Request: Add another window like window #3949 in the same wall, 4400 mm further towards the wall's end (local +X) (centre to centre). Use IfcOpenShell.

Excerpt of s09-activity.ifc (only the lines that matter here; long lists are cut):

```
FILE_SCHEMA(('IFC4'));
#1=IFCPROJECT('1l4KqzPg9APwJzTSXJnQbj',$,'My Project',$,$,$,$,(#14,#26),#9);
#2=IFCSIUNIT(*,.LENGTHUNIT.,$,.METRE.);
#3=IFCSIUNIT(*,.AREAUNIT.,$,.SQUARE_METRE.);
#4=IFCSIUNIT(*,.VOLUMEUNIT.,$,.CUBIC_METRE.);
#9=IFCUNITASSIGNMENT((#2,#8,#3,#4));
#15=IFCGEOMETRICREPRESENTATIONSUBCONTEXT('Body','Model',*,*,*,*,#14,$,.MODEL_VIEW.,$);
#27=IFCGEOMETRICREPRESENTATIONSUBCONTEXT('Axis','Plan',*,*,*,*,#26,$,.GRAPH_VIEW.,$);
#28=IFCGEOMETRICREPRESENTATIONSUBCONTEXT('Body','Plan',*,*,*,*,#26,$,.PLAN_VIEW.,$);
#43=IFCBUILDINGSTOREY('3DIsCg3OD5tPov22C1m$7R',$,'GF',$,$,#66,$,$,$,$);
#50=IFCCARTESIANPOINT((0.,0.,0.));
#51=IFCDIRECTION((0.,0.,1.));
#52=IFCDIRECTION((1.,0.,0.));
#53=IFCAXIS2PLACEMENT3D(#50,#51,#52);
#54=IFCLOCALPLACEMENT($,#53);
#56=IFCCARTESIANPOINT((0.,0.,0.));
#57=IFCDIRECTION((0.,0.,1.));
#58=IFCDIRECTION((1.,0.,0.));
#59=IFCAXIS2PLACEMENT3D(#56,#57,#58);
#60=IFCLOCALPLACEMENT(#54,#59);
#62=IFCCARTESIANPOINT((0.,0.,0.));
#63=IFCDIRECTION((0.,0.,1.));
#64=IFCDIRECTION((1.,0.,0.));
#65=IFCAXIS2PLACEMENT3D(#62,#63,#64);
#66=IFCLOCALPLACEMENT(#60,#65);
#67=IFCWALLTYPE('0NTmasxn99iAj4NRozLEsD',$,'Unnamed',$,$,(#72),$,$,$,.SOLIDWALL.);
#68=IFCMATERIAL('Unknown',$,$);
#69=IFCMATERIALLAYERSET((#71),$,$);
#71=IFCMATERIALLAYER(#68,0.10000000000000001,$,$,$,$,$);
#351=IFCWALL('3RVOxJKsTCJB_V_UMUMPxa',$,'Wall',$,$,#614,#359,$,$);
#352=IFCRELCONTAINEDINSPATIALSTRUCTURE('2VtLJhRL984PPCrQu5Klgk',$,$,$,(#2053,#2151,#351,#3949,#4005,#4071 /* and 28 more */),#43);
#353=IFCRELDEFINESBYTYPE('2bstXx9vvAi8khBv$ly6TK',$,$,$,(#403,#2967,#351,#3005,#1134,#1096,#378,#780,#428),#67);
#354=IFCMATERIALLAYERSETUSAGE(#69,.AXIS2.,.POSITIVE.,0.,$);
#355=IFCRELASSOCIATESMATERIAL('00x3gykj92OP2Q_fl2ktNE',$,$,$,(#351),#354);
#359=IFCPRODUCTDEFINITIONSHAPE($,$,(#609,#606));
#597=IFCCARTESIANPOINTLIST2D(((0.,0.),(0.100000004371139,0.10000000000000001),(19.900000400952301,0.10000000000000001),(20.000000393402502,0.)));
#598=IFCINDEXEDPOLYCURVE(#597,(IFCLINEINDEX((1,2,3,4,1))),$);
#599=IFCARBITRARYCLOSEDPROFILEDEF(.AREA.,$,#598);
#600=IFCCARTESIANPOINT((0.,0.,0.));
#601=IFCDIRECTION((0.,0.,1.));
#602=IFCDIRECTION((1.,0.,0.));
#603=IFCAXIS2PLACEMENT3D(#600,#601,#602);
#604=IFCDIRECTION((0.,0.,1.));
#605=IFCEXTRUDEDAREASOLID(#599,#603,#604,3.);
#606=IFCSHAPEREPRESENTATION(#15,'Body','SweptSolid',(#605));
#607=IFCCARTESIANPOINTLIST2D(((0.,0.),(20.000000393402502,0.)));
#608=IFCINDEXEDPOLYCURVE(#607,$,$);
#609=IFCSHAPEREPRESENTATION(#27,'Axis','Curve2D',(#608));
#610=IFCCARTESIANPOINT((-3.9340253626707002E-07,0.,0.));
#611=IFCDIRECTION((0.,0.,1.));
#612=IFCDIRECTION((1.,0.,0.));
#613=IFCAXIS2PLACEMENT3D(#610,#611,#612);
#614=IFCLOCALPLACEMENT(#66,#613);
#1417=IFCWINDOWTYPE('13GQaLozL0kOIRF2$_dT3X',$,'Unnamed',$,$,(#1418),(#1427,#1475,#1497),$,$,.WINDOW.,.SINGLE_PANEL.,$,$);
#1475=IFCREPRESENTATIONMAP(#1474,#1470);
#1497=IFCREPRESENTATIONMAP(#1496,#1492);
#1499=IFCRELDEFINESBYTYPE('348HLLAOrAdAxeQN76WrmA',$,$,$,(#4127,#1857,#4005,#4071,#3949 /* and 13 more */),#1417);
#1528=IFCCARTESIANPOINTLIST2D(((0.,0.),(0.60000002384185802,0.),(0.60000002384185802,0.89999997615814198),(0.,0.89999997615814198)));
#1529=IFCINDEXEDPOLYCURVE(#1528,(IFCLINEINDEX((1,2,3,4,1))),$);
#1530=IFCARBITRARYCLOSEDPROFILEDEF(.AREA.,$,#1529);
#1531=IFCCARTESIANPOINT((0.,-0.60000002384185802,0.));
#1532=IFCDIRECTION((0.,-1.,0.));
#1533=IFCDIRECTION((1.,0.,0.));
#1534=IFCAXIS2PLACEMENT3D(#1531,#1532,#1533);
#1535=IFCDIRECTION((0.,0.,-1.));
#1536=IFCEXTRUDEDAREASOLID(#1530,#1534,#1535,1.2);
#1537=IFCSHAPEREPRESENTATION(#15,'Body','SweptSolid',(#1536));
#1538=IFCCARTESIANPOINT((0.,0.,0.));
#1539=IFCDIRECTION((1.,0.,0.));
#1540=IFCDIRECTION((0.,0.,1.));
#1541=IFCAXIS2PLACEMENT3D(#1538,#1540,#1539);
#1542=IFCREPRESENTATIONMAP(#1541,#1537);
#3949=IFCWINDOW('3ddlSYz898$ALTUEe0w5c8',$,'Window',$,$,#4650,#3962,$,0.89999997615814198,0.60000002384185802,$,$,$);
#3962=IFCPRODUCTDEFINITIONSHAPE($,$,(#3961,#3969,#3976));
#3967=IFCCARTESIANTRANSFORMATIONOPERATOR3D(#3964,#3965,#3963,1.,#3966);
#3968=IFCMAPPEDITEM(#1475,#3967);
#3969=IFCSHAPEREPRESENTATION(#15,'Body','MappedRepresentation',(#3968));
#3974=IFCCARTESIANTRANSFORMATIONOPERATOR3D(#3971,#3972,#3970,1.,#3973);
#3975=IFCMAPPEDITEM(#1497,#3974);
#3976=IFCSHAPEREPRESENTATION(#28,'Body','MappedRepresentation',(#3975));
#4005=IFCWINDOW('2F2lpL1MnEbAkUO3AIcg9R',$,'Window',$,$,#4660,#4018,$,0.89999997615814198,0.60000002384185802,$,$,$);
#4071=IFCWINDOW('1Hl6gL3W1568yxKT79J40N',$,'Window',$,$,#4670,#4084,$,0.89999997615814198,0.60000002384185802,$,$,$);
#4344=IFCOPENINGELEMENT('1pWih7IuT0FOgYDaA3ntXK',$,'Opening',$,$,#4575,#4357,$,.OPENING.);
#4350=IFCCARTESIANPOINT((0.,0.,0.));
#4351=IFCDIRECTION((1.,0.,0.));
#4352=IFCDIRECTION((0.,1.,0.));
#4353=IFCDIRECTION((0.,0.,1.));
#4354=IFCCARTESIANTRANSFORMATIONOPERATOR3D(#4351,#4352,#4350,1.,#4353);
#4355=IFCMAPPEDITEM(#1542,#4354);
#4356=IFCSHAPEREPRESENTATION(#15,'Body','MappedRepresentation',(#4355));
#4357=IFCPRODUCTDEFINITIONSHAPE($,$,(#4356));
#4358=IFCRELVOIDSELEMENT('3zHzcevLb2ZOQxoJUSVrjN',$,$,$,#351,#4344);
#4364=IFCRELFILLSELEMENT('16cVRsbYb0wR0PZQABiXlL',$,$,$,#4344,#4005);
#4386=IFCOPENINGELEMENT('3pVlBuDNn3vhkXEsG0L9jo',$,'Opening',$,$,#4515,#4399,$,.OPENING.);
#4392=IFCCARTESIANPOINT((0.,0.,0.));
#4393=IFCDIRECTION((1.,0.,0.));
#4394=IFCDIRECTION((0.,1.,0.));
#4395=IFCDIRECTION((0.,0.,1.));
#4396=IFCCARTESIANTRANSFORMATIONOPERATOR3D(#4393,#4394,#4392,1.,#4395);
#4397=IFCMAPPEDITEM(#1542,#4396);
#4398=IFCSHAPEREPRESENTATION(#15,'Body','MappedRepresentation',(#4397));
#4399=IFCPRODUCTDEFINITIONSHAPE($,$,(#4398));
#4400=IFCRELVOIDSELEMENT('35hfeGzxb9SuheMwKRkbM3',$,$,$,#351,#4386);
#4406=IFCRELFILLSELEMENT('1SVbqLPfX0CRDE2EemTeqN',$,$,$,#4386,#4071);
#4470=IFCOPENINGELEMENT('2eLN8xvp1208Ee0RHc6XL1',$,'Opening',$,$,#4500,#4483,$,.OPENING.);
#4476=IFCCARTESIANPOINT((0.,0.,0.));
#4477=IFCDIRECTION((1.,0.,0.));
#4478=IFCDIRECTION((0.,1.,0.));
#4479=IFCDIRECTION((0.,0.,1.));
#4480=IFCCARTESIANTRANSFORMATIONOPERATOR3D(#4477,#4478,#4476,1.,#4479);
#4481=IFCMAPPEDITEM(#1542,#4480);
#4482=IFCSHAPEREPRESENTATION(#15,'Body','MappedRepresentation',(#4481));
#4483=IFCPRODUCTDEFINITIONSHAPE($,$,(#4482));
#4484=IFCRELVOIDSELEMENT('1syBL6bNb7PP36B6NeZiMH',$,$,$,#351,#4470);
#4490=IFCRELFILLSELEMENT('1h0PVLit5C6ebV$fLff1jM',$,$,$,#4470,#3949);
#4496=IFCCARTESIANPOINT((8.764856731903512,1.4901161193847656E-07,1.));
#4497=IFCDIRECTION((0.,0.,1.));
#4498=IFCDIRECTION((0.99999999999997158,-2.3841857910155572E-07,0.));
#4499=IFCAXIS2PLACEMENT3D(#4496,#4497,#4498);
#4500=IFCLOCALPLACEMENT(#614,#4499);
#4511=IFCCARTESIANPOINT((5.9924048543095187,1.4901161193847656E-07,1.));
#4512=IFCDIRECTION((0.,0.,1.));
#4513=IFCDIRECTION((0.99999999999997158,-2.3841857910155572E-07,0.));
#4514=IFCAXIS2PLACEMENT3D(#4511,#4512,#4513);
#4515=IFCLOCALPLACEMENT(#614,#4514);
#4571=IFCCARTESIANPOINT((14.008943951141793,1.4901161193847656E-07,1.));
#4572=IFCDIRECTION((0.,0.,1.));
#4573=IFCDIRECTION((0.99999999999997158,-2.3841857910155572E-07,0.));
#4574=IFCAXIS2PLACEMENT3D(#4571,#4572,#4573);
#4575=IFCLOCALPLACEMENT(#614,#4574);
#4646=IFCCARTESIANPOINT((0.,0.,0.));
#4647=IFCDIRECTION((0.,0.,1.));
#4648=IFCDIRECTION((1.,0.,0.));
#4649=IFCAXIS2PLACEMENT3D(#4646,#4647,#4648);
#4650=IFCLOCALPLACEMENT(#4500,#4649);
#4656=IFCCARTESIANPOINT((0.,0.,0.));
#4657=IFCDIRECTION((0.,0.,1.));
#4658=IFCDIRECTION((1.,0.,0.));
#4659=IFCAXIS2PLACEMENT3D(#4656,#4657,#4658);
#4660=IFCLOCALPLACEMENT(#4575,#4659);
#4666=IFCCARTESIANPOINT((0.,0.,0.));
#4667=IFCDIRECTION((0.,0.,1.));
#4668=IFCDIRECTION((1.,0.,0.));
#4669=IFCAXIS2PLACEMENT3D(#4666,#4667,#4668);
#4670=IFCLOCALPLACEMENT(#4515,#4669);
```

```python
import ifcopenshell
import ifcopenshell.api.feature
import ifcopenshell.api.geometry
import ifcopenshell.api.root
import ifcopenshell.geom
import ifcopenshell.util.element
import ifcopenshell.util.placement
import ifcopenshell.util.shape
import ifcopenshell.util.unit

model = ifcopenshell.open("s09-activity.ifc")
unit_scale = ifcopenshell.util.unit.calculate_unit_scale(model)
settings = ifcopenshell.geom.settings()


def volume(element):
    """Net volume in cubic metres, openings subtracted."""
    shape = ifcopenshell.geom.create_shape(settings, element)
    return ifcopenshell.util.shape.get_volume(shape.geometry)


window = model.by_id(3949)
opening = window.FillsVoids[0].RelatingOpeningElement
wall = opening.VoidsElements[0].RelatingBuildingElement
before = volume(wall)
shift = ifcopenshell.util.placement.get_local_placement(wall.ObjectPlacement)[:3, 0] * 4.4 / unit_scale

# copy_class copies the void relationship, type, container and properties, but no geometry.
new_opening = ifcopenshell.api.root.copy_class(model, product=opening)
new_opening.Representation = ifcopenshell.util.element.copy_deep(
    model, opening.Representation, exclude=["IfcGeometricRepresentationContext", "IfcRepresentationMap"]
)
new_window = ifcopenshell.api.root.copy_class(model, product=window)
new_window.Representation = ifcopenshell.util.element.copy_deep(
    model, window.Representation, exclude=["IfcGeometricRepresentationContext", "IfcRepresentationMap"]
)
ifcopenshell.api.feature.add_filling(model, opening=new_opening, element=new_window)

for old, new in ((opening, new_opening), (window, new_window)):
    matrix = ifcopenshell.util.placement.get_local_placement(old.ObjectPlacement)
    matrix[:3, 3] += shift
    ifcopenshell.api.geometry.edit_object_placement(model, product=new, matrix=matrix, is_si=False)

after = volume(wall)

print(f"wall volume {before:.3f} -> {after:.3f} m3")

model.write("s09-activity_rev.ifc")
```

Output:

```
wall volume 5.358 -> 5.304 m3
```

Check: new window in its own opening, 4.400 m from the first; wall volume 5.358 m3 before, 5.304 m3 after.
